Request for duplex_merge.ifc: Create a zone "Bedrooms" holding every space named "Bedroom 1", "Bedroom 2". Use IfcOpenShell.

First a look at what the model holds.

```python
import ifcopenshell

model = ifcopenshell.open("duplex_merge.ifc")
print(model.schema)
seen = {}
for space in model.by_type("IfcSpace"):
    seen[space.LongName] = seen.get(space.LongName, 0) + 1
for name, count in sorted(seen.items(), key=str):
    print(count, "x", name)
print("zones:", [z.Name for z in model.by_type("IfcZone")][:20])
```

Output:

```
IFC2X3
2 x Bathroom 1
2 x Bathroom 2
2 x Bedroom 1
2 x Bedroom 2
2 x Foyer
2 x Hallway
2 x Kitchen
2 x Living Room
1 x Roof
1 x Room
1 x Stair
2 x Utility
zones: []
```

```python
import ifcopenshell
import ifcopenshell.api.group
import ifcopenshell.api.root

model = ifcopenshell.open("duplex_merge.ifc")

names = {"Bedroom 1", "Bedroom 2"}
spaces = [s for s in model.by_type("IfcSpace") if s.LongName in names]

zone = ifcopenshell.api.root.create_entity(model, ifc_class="IfcZone", name="Bedrooms")
ifcopenshell.api.group.assign_group(model, products=spaces, group=zone)
print(len(spaces), "spaces in", zone.Name)

model.write("duplex_merge_edited.ifc")
```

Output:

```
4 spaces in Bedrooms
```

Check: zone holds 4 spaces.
